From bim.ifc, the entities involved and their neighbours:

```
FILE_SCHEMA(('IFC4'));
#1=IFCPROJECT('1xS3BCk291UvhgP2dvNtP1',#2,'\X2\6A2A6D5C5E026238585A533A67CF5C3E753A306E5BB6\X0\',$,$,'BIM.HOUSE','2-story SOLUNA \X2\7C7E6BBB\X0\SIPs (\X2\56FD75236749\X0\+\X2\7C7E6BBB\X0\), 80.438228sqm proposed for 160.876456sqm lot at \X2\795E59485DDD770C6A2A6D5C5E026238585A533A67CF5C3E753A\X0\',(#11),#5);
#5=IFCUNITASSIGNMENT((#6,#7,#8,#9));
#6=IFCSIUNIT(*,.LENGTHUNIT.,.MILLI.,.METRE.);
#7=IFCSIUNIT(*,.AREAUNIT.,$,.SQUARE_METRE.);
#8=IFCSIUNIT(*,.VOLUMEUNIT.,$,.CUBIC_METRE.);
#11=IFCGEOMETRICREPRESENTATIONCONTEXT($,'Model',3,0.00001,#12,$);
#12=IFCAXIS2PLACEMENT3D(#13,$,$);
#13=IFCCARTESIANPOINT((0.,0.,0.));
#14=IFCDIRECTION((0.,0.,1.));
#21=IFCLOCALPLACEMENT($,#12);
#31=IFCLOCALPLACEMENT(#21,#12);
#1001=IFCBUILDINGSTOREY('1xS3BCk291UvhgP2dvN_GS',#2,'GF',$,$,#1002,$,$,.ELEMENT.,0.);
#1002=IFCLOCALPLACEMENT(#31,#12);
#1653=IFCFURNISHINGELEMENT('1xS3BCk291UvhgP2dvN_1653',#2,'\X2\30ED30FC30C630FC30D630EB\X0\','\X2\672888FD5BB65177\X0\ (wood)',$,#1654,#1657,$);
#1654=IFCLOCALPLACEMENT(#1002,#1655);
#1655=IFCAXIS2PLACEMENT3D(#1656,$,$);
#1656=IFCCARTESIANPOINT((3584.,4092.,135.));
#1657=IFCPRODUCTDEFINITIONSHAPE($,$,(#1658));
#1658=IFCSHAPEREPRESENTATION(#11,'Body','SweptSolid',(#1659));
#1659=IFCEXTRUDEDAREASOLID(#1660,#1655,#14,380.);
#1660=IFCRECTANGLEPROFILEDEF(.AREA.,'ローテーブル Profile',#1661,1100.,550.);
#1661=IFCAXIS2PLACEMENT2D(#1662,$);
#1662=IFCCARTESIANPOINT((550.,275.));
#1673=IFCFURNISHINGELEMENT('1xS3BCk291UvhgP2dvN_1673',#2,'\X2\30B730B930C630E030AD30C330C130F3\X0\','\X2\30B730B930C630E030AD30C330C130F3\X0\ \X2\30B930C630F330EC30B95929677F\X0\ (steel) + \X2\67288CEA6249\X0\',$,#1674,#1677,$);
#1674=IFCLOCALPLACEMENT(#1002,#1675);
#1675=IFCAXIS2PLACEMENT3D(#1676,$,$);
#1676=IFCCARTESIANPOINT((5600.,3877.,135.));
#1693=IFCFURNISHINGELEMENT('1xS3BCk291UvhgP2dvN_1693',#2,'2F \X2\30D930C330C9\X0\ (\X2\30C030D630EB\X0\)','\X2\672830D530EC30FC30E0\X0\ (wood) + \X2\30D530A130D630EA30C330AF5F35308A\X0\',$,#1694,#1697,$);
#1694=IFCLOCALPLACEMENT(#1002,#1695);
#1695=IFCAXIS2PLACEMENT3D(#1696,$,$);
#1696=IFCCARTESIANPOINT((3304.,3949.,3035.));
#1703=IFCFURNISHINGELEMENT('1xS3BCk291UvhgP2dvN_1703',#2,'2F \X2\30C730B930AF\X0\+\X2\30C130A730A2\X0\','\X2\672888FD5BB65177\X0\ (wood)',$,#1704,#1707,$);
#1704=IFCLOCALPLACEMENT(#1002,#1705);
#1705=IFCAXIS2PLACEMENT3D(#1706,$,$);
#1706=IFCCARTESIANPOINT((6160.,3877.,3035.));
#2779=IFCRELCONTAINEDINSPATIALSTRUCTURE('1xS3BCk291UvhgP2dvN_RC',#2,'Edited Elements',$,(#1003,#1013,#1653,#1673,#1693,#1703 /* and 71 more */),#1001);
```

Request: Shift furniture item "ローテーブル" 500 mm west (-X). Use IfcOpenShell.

```python
import ifcopenshell
import ifcopenshell.api.geometry
import ifcopenshell.util.placement

model = ifcopenshell.open("bim.ifc")

item = model.by_guid("1xS3BCk291UvhgP2dvN_1653")
matrix = ifcopenshell.util.placement.get_local_placement(item.ObjectPlacement)
matrix[0, 3] -= 500.0
ifcopenshell.api.geometry.edit_object_placement(model, product=item, matrix=matrix, is_si=False)

print(ifcopenshell.util.placement.get_local_placement(item.ObjectPlacement).round(3) + 0.0)

model.write("bim-out.ifc")
```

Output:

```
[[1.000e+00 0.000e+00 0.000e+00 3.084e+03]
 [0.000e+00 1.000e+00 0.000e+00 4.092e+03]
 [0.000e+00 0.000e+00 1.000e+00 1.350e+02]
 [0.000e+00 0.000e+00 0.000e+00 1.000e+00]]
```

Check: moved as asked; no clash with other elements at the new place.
